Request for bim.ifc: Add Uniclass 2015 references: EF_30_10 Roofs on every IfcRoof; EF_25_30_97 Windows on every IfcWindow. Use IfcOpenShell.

First a look at what the model holds.

```python
import ifcopenshell

model = ifcopenshell.open("bim.ifc")
print(model.schema)
print("classifications:", [c.Name for c in model.by_type("IfcClassification")])
for ifc_class in ("IfcDoor", "IfcRoof", "IfcStair", "IfcWall", "IfcWindow"):
    print(ifc_class, len(model.by_type(ifc_class)))
```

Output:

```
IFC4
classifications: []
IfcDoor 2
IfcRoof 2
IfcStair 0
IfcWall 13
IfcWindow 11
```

```python
import ifcopenshell
import ifcopenshell.api.classification

model = ifcopenshell.open("bim.ifc")

system = ifcopenshell.api.classification.add_classification(model, classification="Uniclass 2015")

codes = {
    "IfcRoof": ("EF_30_10", "Roofs"),
    "IfcWindow": ("EF_25_30_97", "Windows"),
}
for ifc_class, (code, name) in codes.items():
    products = model.by_type(ifc_class)
    ifcopenshell.api.classification.add_reference(
        model, products=products, classification=system, identification=code, name=name
    )
    print(code, len(products))

model.write("bim_rev.ifc")
```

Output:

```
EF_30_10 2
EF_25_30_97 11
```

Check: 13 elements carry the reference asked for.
